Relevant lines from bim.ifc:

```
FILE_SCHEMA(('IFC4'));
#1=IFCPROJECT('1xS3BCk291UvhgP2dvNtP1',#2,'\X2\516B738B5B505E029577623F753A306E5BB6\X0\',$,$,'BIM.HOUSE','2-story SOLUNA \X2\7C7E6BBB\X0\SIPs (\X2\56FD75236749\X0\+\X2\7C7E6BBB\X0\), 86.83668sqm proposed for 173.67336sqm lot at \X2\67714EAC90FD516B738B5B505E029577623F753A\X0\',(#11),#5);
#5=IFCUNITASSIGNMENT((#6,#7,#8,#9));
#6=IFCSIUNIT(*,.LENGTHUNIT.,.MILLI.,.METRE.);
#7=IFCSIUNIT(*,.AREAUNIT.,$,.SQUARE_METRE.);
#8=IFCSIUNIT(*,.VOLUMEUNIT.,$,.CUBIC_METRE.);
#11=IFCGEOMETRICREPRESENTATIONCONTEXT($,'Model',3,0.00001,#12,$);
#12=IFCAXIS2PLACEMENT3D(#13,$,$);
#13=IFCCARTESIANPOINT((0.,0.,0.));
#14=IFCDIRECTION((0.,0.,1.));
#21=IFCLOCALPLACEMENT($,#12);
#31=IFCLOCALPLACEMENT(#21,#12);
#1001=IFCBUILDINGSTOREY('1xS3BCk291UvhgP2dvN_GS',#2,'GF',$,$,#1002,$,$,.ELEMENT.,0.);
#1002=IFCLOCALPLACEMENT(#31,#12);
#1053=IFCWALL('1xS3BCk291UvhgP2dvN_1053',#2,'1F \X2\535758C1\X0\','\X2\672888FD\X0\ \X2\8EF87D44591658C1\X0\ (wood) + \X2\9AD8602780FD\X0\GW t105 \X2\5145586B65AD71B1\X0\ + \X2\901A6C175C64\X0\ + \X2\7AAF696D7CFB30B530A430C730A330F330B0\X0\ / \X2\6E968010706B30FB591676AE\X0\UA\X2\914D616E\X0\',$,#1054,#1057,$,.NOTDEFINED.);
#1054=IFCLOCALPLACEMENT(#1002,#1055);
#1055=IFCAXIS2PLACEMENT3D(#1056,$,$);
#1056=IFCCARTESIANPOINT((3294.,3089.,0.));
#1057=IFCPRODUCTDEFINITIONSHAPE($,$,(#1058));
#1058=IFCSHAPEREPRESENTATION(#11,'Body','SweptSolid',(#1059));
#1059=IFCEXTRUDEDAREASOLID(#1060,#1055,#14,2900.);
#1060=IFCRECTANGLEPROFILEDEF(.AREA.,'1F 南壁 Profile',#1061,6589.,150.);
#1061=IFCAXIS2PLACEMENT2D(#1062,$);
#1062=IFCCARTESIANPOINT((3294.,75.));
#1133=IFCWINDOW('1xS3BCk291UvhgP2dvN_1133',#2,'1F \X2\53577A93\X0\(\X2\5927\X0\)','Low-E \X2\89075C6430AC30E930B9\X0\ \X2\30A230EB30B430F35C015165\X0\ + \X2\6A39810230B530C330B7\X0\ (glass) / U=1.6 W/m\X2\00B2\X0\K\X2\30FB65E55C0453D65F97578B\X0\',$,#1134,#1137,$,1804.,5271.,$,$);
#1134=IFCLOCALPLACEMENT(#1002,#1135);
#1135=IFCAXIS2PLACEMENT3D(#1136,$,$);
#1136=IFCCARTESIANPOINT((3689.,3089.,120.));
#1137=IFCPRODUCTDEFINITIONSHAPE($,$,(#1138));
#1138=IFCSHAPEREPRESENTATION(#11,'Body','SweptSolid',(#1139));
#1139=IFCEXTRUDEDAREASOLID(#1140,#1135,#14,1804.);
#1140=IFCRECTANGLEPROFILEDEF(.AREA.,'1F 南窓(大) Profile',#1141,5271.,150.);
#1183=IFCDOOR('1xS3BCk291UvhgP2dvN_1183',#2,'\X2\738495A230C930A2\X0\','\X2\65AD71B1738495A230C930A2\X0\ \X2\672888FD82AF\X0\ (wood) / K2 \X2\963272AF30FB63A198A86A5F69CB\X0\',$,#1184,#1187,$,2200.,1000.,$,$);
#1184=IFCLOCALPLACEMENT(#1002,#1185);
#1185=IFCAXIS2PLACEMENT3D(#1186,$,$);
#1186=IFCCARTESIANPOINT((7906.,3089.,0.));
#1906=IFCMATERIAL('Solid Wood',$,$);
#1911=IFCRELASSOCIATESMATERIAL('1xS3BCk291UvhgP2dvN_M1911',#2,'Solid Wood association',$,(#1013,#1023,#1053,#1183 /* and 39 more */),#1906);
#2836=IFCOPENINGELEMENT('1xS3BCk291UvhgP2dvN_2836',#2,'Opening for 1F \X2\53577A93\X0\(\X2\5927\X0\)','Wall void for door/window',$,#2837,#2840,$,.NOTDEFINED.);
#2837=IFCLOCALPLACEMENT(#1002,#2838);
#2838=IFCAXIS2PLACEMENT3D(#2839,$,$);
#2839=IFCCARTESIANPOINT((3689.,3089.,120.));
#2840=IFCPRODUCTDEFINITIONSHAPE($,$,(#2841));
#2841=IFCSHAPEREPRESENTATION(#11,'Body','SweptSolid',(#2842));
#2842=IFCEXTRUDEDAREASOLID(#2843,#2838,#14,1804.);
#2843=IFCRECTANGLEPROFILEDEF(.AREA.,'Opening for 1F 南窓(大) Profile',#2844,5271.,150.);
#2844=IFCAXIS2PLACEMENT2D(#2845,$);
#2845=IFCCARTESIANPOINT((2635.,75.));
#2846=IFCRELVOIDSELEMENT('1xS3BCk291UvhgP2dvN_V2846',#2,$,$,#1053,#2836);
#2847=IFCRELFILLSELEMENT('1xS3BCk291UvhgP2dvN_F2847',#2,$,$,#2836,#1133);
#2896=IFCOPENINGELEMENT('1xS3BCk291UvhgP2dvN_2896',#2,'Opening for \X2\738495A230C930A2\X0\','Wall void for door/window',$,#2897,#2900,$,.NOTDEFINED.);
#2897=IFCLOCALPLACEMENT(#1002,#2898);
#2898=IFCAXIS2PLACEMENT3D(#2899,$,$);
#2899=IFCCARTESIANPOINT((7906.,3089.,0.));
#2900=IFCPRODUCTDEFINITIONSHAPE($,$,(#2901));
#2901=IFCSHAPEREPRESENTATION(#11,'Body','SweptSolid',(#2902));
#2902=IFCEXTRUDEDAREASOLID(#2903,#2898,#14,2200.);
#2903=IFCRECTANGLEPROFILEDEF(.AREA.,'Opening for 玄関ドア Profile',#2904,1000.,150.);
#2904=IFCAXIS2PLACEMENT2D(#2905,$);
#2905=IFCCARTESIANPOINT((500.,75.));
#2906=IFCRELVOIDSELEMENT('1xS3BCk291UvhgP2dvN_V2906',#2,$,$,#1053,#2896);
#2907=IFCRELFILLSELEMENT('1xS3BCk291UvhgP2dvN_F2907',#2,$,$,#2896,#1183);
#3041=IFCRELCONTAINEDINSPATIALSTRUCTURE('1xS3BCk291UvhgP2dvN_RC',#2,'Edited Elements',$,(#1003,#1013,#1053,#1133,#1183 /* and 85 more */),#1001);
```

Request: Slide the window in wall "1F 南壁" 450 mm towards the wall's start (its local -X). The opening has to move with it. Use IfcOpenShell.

```python
import ifcopenshell
import ifcopenshell.api.geometry
import ifcopenshell.util.placement

model = ifcopenshell.open("bim.ifc")

window = model.by_id(1133)
opening = window.FillsVoids[0].RelatingOpeningElement
wall = opening.VoidsElements[0].RelatingBuildingElement

wall_matrix = ifcopenshell.util.placement.get_local_placement(wall.ObjectPlacement)
shift = wall_matrix[:3, 0] * -450.0
before = ifcopenshell.util.placement.get_local_placement(window.ObjectPlacement)[:3, 3].copy()

# The window is not placed relative to its opening, so move both.
for product in (opening, window):
    matrix = ifcopenshell.util.placement.get_local_placement(product.ObjectPlacement)
    matrix[:3, 3] += shift
    ifcopenshell.api.geometry.edit_object_placement(model, product=product, matrix=matrix, is_si=False)

after = ifcopenshell.util.placement.get_local_placement(window.ObjectPlacement)[:3, 3]
print("window moved by", (after - before).round(3) + 0.0)

model.write("bim_updated.ifc")
```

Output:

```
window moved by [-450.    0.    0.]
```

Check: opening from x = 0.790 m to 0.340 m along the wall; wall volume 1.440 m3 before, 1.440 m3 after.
